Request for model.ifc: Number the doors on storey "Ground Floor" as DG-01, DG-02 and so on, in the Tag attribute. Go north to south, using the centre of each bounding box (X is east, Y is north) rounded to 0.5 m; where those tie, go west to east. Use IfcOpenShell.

First a look at what the model holds.

```python
import ifcopenshell
import ifcopenshell.util.element
import ifcopenshell.util.placement

model = ifcopenshell.open("model.ifc")
print(model.schema)
storey = next(s for s in model.by_type("IfcBuildingStorey") if s.Name == "Ground Floor")
doors = [e for e in ifcopenshell.util.element.get_decomposition(storey) if e.is_a("IfcDoor")]
for e in sorted(doors, key=lambda e: e.id()):
    origin = ifcopenshell.util.placement.get_local_placement(e.ObjectPlacement)[:3, 3]
    print(e.id(), e.Tag, e.Name, origin.round(2) + 0.0, sep=" | ")
```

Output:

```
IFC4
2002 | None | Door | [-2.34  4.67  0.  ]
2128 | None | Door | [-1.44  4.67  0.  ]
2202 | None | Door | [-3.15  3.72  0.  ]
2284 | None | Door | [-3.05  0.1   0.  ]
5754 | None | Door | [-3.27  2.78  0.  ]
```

```python
import ifcopenshell
import ifcopenshell.geom
import ifcopenshell.util.element
import ifcopenshell.util.shape

model = ifcopenshell.open("model.ifc")
settings = ifcopenshell.geom.settings()
settings.set("use-world-coords", True)


def centre(element):
    shape = ifcopenshell.geom.create_shape(settings, element)
    return ifcopenshell.util.shape.get_bbox_centroid(shape.geometry)


storey = next(s for s in model.by_type("IfcBuildingStorey") if s.Name == "Ground Floor")
doors = [e for e in ifcopenshell.util.element.get_decomposition(storey) if e.is_a("IfcDoor")]

# Insertion points can sit at a corner or the storey origin, so sort by the geometry (in metres).
centres = {e: centre(e) for e in doors}
doors.sort(key=lambda e: (-round(centres[e][1] / 0.5), centres[e][0]))

for i, e in enumerate(doors, start=1):
    number = f"DG-{i:02d}"
    e.Tag = number
    print(e.id(), number)

model.write("model_v2.ifc")
```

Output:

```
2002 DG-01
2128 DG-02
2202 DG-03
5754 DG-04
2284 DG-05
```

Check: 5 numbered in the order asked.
